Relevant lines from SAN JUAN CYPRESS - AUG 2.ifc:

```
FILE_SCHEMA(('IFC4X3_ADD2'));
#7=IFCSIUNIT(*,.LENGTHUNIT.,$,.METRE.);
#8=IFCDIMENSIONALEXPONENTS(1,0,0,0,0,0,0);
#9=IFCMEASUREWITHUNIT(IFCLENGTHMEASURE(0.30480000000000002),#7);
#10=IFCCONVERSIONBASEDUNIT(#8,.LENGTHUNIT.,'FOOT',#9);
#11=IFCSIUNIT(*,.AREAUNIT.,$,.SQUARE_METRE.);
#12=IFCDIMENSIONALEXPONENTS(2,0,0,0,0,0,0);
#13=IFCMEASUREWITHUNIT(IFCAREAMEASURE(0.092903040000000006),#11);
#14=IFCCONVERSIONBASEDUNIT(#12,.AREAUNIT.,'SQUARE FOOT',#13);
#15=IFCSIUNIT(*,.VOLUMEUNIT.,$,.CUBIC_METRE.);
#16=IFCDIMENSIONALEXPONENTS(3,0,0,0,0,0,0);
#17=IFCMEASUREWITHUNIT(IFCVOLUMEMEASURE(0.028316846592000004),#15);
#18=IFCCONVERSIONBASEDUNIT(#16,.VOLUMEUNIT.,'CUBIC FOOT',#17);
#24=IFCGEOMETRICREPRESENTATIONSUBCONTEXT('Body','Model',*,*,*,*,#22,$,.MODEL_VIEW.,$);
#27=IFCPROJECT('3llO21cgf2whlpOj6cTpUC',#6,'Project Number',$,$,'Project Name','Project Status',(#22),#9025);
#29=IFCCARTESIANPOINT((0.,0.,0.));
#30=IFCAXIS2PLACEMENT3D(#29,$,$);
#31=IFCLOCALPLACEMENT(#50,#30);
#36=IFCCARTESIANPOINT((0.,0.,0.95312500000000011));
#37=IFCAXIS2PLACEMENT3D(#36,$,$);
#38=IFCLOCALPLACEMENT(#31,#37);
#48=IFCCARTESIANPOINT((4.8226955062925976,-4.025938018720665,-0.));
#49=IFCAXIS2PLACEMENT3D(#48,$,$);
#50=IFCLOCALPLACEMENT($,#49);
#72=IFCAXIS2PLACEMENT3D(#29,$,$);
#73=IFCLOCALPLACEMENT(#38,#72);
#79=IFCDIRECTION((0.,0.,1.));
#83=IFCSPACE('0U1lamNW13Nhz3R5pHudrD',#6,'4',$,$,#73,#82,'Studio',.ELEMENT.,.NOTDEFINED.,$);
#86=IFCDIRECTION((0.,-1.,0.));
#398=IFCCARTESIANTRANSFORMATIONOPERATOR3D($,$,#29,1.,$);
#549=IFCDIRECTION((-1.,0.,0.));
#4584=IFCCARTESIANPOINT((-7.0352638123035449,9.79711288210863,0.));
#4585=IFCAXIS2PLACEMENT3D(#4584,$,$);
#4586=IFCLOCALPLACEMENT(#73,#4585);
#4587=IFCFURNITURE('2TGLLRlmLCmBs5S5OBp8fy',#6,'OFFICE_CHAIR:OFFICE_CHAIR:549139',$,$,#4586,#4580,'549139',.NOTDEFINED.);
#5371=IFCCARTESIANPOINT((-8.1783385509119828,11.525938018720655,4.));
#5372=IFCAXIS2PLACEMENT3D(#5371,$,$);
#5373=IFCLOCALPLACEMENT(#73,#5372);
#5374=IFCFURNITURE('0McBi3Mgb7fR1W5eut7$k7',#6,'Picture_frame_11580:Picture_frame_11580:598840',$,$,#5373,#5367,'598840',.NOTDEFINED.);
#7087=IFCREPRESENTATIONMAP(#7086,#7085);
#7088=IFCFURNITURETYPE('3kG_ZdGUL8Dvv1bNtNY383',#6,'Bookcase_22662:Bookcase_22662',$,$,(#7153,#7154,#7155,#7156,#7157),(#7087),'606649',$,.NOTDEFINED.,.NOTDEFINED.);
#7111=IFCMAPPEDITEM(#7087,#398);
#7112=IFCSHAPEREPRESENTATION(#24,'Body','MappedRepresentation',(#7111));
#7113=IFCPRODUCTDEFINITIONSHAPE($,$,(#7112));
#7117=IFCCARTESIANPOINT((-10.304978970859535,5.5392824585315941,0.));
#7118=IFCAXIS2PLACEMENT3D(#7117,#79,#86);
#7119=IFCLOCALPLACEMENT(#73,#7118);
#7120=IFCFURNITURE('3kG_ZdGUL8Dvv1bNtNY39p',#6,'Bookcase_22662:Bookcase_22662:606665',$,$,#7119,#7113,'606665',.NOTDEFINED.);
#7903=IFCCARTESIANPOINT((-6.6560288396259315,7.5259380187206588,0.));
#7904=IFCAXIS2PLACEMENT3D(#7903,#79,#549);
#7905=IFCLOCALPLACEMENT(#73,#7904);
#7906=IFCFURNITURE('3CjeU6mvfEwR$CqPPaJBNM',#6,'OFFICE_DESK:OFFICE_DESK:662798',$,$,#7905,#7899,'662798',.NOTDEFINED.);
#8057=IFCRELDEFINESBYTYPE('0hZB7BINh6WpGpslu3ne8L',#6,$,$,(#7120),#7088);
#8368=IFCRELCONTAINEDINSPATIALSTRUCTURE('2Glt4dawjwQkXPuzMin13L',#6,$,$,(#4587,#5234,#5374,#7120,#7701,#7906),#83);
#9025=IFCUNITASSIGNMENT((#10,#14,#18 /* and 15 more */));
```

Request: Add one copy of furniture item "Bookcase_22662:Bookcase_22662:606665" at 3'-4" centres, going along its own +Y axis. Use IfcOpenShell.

```python
import ifcopenshell
import ifcopenshell.api.geometry
import ifcopenshell.api.root
import ifcopenshell.util.element
import ifcopenshell.util.placement
import ifcopenshell.util.unit

model = ifcopenshell.open("SAN JUAN CYPRESS - AUG 2.ifc")
unit_scale = ifcopenshell.util.unit.calculate_unit_scale(model)


def reuse_history(source, copy):
    """copy_class also copies each property set's owner history, people and application; keep the originals."""
    for rel in copy.IsDefinedBy:
        if rel.is_a("IfcRelDefinesByProperties") and (history := rel.RelatingPropertyDefinition.OwnerHistory):
            rel.RelatingPropertyDefinition.OwnerHistory = source.OwnerHistory
            ifcopenshell.util.element.remove_deep2(model, history)


source = model.by_id(7120)
base = ifcopenshell.util.placement.get_local_placement(source.ObjectPlacement)
step = base[:3, 1] * 40 * 0.0254 / unit_scale

for i in range(1, 2):
    copy = ifcopenshell.api.root.copy_class(model, product=source)
    copy.Representation = ifcopenshell.util.element.copy_deep(
        model, source.Representation, exclude=["IfcGeometricRepresentationContext", "IfcRepresentationMap"]
    )
    copy.Name = "Bookcase_22662:Bookcase_22662"
    copy.Tag = None
    reuse_history(source, copy)
    matrix = base.copy()
    matrix[:3, 3] += i * step
    print("added at", matrix[:3, 3].round(3) + 0.0)
    ifcopenshell.api.geometry.edit_object_placement(model, product=copy, matrix=matrix, is_si=False)

model.write("SAN JUAN CYPRESS - AUG 2_v2.ifc")
```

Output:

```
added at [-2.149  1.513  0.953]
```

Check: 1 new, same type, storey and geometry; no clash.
